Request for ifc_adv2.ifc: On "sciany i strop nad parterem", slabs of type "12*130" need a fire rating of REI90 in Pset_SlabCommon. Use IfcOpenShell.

First a look at what the model holds.

```python
import ifcopenshell
import ifcopenshell.util.element

model = ifcopenshell.open("ifc_adv2.ifc")
print(model.schema)
storey = next(s for s in model.by_type("IfcBuildingStorey") if s.Name == "sciany i strop nad parterem")
slabs = [e for e in ifcopenshell.util.element.get_decomposition(storey) if e.is_a("IfcSlab")]
seen = {}
for e in slabs:
    element_type = ifcopenshell.util.element.get_type(e)
    key = (element_type.Name if element_type != e and element_type else None, ifcopenshell.util.element.get_pset(e, "Pset_SlabCommon", "FireRating"))
    seen[key] = seen.get(key, 0) + 1
for (name, value), count in sorted(seen.items(), key=str):
    print(count, "x", name, "|", value)
```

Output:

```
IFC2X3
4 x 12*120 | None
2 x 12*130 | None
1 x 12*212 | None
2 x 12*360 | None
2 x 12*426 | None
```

```python
import ifcopenshell
import ifcopenshell.api.pset
import ifcopenshell.util.element

model = ifcopenshell.open("ifc_adv2.ifc")

storey = next(s for s in model.by_type("IfcBuildingStorey") if s.Name == "sciany i strop nad parterem")
slabs = [e for e in ifcopenshell.util.element.get_decomposition(storey) if e.is_a("IfcSlab")]

count = 0
for e in slabs:
    element_type = ifcopenshell.util.element.get_type(e)
    if element_type in (None, e) or element_type.Name != "12*130":
        continue
    # add_pset returns the element's existing set when there is one.
    pset = ifcopenshell.api.pset.add_pset(model, product=e, name="Pset_SlabCommon")
    ifcopenshell.api.pset.edit_pset(model, pset=pset, properties={"FireRating": "REI90"})
    count += 1

print(count, "slabs updated")

model.write("ifc_adv2_v2.ifc")
```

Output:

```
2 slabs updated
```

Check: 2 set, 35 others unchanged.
